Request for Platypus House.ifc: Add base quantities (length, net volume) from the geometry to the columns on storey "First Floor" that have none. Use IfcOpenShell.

First a look at what the model holds.

```python
import ifcopenshell
import ifcopenshell.util.element
import ifcopenshell.util.unit

model = ifcopenshell.open("Platypus House.ifc")
print(model.schema)
for unit_type in ("LENGTHUNIT", "AREAUNIT", "VOLUMEUNIT"):
    print(unit_type, ifcopenshell.util.unit.calculate_unit_scale(model, unit_type))
storey = next(s for s in model.by_type("IfcBuildingStorey") if s.Name == "First Floor")
columns = [e for e in ifcopenshell.util.element.get_decomposition(storey) if e.is_a("IfcColumn")]
for e in sorted(columns, key=lambda e: e.id()):
    print(e.id(), e.is_a(), e.Name, list(ifcopenshell.util.element.get_psets(e, qtos_only=True)), sep=" | ")
```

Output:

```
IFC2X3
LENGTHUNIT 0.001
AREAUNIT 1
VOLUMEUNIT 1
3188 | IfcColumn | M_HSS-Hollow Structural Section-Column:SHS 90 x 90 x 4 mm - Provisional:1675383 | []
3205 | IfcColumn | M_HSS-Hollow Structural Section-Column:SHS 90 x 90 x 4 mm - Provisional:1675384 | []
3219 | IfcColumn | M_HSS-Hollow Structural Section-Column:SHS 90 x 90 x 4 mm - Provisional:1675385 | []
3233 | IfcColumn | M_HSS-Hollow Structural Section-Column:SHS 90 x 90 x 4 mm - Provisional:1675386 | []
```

```python
import ifcopenshell
import ifcopenshell.api.pset
import ifcopenshell.geom
import ifcopenshell.util.element
import ifcopenshell.util.shape
import ifcopenshell.util.unit

model = ifcopenshell.open("Platypus House.ifc")
unit_scale = ifcopenshell.util.unit.calculate_unit_scale(model)
volume_scale = ifcopenshell.util.unit.calculate_unit_scale(model, "VOLUMEUNIT")
settings = ifcopenshell.geom.settings()

storey = next(s for s in model.by_type("IfcBuildingStorey") if s.Name == "First Floor")
columns = [e for e in ifcopenshell.util.element.get_decomposition(storey) if e.is_a("IfcColumn")]

for e in sorted(columns, key=lambda e: e.id()):
    if ifcopenshell.util.element.get_psets(e, qtos_only=True, should_inherit=False):
        continue
    # Geometry comes back in metres, in the element's own axes.
    shape = ifcopenshell.geom.create_shape(settings, e)
    values = {
        "Length": ifcopenshell.util.shape.get_z(shape.geometry) / unit_scale,
        "NetVolume": ifcopenshell.util.shape.get_volume(shape.geometry) / volume_scale,
    }
    qto = ifcopenshell.api.pset.add_qto(model, product=e, name="BaseQuantities")
    ifcopenshell.api.pset.edit_qto(model, qto=qto, properties=values)
    print(e.id(), {k: round(v, 3) for k, v in values.items()})

model.write("Platypus House_rev.ifc")
```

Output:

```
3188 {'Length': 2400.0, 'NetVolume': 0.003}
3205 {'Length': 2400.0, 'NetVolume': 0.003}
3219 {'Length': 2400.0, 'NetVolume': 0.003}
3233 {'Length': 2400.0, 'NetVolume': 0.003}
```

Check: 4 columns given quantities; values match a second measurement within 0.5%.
